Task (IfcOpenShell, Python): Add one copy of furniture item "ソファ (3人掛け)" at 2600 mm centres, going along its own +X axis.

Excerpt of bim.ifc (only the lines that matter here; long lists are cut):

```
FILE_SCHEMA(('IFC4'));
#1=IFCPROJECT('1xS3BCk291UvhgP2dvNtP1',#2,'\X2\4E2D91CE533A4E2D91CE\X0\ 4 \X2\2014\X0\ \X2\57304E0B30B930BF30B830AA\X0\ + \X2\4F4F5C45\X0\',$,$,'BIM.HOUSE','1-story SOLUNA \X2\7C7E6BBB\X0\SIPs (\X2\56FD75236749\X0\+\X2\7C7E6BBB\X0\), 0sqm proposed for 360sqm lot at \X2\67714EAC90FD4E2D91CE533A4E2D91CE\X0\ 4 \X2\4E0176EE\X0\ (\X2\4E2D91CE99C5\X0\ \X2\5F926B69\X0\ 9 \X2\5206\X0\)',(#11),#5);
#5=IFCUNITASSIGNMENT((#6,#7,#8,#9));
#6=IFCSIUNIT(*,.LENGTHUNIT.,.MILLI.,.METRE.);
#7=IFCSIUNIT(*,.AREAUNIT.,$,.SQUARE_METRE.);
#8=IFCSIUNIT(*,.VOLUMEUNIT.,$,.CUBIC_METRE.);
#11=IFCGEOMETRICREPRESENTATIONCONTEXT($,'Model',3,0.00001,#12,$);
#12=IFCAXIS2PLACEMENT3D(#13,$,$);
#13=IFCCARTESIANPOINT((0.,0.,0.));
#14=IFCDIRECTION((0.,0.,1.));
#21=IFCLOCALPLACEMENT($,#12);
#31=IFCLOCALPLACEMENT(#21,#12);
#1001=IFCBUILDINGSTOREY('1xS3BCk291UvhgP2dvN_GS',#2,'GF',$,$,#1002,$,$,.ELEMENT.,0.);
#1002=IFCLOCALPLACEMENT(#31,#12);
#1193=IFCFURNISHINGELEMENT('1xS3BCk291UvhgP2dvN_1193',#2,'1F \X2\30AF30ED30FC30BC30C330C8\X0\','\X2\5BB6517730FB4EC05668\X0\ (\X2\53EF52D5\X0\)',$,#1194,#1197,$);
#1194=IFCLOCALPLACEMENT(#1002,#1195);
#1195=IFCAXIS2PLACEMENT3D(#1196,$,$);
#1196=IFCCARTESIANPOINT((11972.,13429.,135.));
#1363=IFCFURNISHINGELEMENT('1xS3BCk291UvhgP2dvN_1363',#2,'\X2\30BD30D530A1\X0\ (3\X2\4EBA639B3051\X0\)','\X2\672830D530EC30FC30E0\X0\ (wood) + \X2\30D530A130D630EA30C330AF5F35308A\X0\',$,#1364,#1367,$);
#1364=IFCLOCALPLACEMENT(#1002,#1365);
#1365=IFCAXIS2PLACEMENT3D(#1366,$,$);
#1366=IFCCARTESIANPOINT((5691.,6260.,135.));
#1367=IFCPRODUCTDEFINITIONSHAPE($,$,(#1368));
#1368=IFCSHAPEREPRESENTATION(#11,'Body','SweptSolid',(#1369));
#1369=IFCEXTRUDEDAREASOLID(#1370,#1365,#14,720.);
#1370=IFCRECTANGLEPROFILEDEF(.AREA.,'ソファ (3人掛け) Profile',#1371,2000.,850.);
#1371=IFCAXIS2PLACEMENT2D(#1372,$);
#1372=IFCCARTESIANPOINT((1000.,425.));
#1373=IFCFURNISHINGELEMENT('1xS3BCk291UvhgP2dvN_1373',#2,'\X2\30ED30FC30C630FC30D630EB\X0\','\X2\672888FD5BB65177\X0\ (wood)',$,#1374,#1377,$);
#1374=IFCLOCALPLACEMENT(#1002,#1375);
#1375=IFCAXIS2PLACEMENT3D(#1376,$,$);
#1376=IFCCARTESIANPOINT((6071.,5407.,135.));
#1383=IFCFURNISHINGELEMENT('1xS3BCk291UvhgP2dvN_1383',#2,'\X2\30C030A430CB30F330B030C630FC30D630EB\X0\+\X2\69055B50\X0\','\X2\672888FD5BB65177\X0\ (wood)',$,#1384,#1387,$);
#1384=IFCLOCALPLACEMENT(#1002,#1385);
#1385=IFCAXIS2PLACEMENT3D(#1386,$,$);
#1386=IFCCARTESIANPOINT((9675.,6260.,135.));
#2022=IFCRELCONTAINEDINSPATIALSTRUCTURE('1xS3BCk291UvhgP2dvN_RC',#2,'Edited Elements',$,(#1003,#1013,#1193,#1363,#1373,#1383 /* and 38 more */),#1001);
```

```python
import ifcopenshell
import ifcopenshell.api.geometry
import ifcopenshell.api.root
import ifcopenshell.util.element
import ifcopenshell.util.placement

model = ifcopenshell.open("bim.ifc")


def reuse_history(source, copy):
    """copy_class also copies each property set's owner history, people and application; keep the originals."""
    for rel in copy.IsDefinedBy:
        if rel.is_a("IfcRelDefinesByProperties") and (history := rel.RelatingPropertyDefinition.OwnerHistory):
            rel.RelatingPropertyDefinition.OwnerHistory = source.OwnerHistory
            ifcopenshell.util.element.remove_deep2(model, history)


source = model.by_guid("1xS3BCk291UvhgP2dvN_1363")
base = ifcopenshell.util.placement.get_local_placement(source.ObjectPlacement)
step = base[:3, 0] * 2600.0

for i in range(1, 2):
    copy = ifcopenshell.api.root.copy_class(model, product=source)
    copy.Representation = ifcopenshell.util.element.copy_deep(
        model, source.Representation, exclude=["IfcGeometricRepresentationContext", "IfcRepresentationMap"]
    )
    reuse_history(source, copy)
    matrix = base.copy()
    matrix[:3, 3] += i * step
    print("added at", matrix[:3, 3].round(3) + 0.0)
    ifcopenshell.api.geometry.edit_object_placement(model, product=copy, matrix=matrix, is_si=False)

model.write("bim-out.ifc")
```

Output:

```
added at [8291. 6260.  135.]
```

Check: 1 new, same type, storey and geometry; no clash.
